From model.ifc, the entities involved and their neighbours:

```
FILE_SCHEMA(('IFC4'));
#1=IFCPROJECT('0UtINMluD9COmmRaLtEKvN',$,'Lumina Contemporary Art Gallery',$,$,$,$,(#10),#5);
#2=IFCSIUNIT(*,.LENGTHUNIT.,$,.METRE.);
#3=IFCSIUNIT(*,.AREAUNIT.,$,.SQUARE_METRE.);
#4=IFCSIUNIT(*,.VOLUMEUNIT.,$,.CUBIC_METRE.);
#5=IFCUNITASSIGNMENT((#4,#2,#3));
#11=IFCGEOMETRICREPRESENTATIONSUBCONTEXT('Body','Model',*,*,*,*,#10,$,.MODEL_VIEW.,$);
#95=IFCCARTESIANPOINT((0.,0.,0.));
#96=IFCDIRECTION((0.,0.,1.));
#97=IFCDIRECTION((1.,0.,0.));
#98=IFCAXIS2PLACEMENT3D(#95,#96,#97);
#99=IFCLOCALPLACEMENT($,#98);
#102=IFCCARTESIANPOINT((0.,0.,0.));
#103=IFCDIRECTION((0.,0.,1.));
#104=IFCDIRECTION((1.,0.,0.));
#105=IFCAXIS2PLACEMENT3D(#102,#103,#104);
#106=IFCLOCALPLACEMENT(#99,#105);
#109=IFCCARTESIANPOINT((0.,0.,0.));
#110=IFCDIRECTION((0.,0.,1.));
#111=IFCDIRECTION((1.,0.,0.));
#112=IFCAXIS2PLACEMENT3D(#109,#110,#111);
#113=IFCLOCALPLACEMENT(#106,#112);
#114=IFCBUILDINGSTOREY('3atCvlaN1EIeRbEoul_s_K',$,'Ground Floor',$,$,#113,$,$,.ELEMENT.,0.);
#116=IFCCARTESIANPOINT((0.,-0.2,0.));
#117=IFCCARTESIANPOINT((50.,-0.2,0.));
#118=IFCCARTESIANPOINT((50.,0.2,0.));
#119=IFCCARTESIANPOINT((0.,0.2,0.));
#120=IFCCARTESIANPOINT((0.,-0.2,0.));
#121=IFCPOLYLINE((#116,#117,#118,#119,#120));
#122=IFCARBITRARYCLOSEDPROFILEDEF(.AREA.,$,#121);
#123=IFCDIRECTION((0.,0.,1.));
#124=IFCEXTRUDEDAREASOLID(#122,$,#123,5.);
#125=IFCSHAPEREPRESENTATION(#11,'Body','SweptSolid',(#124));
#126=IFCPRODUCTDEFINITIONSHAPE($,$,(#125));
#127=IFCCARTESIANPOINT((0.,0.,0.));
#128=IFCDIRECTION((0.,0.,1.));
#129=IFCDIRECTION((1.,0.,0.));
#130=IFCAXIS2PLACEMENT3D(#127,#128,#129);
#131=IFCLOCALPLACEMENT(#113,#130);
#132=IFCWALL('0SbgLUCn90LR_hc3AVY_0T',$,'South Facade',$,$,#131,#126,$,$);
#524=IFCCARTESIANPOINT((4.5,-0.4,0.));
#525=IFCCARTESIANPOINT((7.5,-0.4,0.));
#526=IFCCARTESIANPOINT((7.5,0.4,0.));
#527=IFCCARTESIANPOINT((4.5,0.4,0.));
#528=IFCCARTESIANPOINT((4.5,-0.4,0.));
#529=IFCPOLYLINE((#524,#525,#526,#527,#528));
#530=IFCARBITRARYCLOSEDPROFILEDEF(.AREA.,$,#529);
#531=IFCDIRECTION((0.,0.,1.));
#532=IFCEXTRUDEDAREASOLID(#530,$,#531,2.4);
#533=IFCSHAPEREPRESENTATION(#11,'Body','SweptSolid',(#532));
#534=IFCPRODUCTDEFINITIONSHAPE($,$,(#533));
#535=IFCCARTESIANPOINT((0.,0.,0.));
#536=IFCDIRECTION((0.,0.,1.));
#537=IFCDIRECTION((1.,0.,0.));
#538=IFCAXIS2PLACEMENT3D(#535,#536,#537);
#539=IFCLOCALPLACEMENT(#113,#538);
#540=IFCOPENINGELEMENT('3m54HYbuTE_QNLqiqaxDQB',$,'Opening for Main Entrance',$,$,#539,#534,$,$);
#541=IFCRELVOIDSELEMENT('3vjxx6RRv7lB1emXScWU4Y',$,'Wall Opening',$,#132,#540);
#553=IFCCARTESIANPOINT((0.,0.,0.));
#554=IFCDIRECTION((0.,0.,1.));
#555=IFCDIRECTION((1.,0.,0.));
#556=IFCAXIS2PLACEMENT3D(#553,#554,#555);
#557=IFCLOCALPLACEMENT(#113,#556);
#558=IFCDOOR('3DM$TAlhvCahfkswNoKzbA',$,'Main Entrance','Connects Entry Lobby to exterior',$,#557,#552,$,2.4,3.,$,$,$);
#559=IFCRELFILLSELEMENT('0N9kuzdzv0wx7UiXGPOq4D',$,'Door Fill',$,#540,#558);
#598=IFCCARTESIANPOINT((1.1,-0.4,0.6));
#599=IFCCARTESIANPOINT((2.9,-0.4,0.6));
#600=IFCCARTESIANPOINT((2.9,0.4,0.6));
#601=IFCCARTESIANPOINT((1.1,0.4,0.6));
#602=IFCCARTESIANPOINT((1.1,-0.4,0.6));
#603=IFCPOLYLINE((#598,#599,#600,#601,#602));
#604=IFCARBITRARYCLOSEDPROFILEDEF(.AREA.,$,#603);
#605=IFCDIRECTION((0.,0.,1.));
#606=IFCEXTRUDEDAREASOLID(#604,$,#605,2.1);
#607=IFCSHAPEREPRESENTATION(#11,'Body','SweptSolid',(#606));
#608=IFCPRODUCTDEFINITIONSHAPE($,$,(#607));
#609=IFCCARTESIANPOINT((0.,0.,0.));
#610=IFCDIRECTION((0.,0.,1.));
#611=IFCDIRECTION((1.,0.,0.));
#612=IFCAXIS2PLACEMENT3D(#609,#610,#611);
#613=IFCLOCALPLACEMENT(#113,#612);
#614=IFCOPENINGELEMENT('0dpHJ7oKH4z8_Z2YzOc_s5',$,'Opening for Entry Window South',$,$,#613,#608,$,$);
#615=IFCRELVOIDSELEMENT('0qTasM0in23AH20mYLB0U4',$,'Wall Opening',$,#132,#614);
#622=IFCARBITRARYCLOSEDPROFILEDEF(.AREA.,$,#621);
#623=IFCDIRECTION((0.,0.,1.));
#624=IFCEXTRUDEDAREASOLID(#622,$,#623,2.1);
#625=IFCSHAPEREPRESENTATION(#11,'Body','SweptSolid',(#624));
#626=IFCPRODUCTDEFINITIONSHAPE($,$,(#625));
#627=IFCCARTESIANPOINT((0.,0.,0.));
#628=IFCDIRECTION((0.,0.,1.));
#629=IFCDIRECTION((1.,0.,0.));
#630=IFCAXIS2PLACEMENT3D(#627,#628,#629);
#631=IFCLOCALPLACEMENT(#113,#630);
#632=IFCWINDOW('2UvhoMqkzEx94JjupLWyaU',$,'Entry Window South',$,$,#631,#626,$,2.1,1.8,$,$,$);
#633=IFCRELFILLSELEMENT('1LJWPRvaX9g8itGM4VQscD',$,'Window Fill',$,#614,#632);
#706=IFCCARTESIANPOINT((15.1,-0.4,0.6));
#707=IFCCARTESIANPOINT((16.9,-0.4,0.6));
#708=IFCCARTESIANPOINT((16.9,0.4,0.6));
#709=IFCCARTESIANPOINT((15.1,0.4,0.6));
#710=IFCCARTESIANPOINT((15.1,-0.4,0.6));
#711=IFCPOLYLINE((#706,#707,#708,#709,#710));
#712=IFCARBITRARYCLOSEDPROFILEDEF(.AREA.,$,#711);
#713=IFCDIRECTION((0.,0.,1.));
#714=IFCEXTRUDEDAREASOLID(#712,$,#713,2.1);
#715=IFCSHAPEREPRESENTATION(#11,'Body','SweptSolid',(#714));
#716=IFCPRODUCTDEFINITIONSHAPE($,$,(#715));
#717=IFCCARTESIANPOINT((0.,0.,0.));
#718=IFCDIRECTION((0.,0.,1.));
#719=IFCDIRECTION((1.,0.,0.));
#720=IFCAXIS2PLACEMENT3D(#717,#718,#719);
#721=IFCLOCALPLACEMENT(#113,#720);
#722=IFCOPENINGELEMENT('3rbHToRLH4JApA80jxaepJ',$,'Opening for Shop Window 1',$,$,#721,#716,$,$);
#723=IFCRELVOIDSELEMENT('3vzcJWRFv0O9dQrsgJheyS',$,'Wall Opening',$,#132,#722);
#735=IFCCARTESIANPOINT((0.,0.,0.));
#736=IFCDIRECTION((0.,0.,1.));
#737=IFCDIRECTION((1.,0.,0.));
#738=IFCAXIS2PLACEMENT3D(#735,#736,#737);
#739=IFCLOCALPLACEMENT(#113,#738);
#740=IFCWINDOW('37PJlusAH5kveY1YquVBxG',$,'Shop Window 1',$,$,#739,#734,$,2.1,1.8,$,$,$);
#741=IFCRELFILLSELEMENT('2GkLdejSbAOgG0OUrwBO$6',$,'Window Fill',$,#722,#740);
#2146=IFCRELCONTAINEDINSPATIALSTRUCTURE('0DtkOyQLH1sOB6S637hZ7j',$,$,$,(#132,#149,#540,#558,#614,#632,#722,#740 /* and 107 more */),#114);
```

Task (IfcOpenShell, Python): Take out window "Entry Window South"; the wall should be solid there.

```python
import ifcopenshell
import ifcopenshell.api.feature
import ifcopenshell.api.root
import ifcopenshell.geom
import ifcopenshell.util.shape

model = ifcopenshell.open("model.ifc")
settings = ifcopenshell.geom.settings()


def volume(element):
    """Net volume in cubic metres, openings subtracted."""
    shape = ifcopenshell.geom.create_shape(settings, element)
    return ifcopenshell.util.shape.get_volume(shape.geometry)


window = model.by_guid("2UvhoMqkzEx94JjupLWyaU")
opening = window.FillsVoids[0].RelatingOpeningElement
wall = opening.VoidsElements[0].RelatingBuildingElement
before = volume(wall)

ifcopenshell.api.root.remove_product(model, product=window)
ifcopenshell.api.feature.remove_feature(model, feature=opening)

after = volume(wall)

print(f"wall volume {before:.3f} -> {after:.3f} m3")

model.write("model-out.ifc")
```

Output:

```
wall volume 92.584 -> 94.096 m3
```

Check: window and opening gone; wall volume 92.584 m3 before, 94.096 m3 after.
